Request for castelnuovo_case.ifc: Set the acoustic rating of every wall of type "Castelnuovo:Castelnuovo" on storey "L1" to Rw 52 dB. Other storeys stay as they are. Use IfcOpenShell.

First a look at what the model holds.

```python
import ifcopenshell
import ifcopenshell.util.element

model = ifcopenshell.open("castelnuovo_case.ifc")
print(model.schema)
storey = next(s for s in model.by_type("IfcBuildingStorey") if s.Name == "L1")
walls = [e for e in ifcopenshell.util.element.get_decomposition(storey) if e.is_a("IfcWall")]
seen = {}
for e in walls:
    element_type = ifcopenshell.util.element.get_type(e)
    key = (element_type.Name if element_type != e and element_type else None, ifcopenshell.util.element.get_pset(e, "Pset_WallCommon", "AcousticRating"))
    seen[key] = seen.get(key, 0) + 1
for (name, value), count in sorted(seen.items(), key=str):
    print(count, "x", name, "|", value)
```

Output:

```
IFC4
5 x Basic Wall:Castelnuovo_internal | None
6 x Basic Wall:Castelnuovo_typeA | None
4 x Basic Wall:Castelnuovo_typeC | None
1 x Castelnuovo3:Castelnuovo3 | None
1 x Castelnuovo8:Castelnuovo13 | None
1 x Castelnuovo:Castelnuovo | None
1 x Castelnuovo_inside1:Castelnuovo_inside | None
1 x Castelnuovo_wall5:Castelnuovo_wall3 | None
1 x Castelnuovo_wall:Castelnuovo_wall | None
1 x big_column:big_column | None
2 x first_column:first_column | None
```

```python
import ifcopenshell
import ifcopenshell.api.pset
import ifcopenshell.util.element

model = ifcopenshell.open("castelnuovo_case.ifc")

storey = next(s for s in model.by_type("IfcBuildingStorey") if s.Name == "L1")
walls = [e for e in ifcopenshell.util.element.get_decomposition(storey) if e.is_a("IfcWall")]

count = 0
for e in walls:
    element_type = ifcopenshell.util.element.get_type(e)
    if element_type in (None, e) or element_type.Name != "Castelnuovo:Castelnuovo":
        continue
    # add_pset returns the element's existing set when there is one.
    pset = ifcopenshell.api.pset.add_pset(model, product=e, name="Pset_WallCommon")
    ifcopenshell.api.pset.edit_pset(model, pset=pset, properties={"AcousticRating": "Rw 52 dB"})
    count += 1

print(count, "walls updated")

model.write("castelnuovo_case_updated.ifc")
```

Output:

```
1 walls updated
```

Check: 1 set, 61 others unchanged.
